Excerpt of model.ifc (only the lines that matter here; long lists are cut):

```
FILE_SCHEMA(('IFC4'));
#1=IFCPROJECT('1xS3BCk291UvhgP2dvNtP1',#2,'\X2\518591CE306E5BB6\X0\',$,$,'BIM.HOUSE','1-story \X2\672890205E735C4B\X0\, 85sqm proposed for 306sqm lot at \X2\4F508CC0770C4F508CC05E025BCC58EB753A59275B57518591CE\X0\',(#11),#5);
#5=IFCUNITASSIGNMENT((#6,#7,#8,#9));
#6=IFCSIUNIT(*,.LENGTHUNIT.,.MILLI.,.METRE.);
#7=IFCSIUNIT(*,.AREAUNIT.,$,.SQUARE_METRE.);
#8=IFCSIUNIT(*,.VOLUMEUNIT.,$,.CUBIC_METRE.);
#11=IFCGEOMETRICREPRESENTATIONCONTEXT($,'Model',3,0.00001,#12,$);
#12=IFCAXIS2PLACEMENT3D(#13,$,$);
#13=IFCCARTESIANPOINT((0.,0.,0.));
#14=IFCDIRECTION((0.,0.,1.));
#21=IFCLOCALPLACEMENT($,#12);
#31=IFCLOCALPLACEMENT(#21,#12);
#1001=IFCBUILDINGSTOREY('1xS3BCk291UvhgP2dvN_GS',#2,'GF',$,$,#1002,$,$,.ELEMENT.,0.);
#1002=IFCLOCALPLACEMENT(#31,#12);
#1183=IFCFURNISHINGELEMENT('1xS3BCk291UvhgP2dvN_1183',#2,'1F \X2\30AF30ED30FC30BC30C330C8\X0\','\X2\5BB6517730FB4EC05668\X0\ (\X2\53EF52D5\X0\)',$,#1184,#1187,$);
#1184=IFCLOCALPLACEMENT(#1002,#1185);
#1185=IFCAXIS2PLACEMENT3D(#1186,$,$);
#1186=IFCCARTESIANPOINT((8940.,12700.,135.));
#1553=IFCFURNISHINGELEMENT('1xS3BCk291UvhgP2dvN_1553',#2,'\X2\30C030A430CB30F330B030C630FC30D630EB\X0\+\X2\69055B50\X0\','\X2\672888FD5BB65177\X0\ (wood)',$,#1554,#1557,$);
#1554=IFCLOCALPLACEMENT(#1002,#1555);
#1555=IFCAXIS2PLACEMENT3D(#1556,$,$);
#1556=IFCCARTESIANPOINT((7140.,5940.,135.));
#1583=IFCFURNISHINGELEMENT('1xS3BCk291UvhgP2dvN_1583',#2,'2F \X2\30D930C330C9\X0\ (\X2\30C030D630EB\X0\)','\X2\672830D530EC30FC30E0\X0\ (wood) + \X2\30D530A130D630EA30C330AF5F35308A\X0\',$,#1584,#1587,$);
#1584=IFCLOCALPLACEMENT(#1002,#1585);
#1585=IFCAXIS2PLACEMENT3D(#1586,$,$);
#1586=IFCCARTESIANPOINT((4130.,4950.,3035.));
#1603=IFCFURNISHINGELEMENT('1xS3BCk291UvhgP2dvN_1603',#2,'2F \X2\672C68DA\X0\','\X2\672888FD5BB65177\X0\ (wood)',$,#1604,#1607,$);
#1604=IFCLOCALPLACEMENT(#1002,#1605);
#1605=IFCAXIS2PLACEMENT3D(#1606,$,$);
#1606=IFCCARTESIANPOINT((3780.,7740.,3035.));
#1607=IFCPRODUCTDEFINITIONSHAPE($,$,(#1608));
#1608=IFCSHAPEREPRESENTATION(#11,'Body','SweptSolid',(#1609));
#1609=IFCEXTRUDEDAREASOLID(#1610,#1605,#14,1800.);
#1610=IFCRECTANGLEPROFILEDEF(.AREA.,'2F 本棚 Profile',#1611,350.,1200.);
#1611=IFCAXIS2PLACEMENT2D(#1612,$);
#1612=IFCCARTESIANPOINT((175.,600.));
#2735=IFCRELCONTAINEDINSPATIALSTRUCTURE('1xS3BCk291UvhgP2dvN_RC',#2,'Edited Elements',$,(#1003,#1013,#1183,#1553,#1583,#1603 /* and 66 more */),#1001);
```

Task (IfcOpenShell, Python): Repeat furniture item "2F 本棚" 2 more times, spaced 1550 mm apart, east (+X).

```python
import numpy as np
import ifcopenshell
import ifcopenshell.api.geometry
import ifcopenshell.api.root
import ifcopenshell.util.element
import ifcopenshell.util.placement

model = ifcopenshell.open("model.ifc")


def reuse_history(source, copy):
    """copy_class also copies each property set's owner history, people and application; keep the originals."""
    for rel in copy.IsDefinedBy:
        if rel.is_a("IfcRelDefinesByProperties") and (history := rel.RelatingPropertyDefinition.OwnerHistory):
            rel.RelatingPropertyDefinition.OwnerHistory = source.OwnerHistory
            ifcopenshell.util.element.remove_deep2(model, history)


source = model.by_guid("1xS3BCk291UvhgP2dvN_1603")
base = ifcopenshell.util.placement.get_local_placement(source.ObjectPlacement)
step = np.array([1.0, 0.0, 0.0]) * 1550.0

for i in range(1, 3):
    copy = ifcopenshell.api.root.copy_class(model, product=source)
    copy.Representation = ifcopenshell.util.element.copy_deep(
        model, source.Representation, exclude=["IfcGeometricRepresentationContext", "IfcRepresentationMap"]
    )
    reuse_history(source, copy)
    matrix = base.copy()
    matrix[:3, 3] += i * step
    print("added at", matrix[:3, 3].round(3) + 0.0)
    ifcopenshell.api.geometry.edit_object_placement(model, product=copy, matrix=matrix, is_si=False)

model.write("model_edited.ifc")
```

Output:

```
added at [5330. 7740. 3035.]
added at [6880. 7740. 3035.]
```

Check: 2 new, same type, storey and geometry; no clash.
